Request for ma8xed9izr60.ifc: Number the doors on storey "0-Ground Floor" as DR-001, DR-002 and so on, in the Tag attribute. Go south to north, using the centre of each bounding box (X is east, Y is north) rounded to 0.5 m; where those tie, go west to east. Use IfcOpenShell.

First a look at what the model holds.

```python
import ifcopenshell
import ifcopenshell.util.element
import ifcopenshell.util.placement

model = ifcopenshell.open("ma8xed9izr60.ifc")
print(model.schema)
storey = next(s for s in model.by_type("IfcBuildingStorey") if s.Name == "0-Ground Floor")
doors = [e for e in ifcopenshell.util.element.get_decomposition(storey) if e.is_a("IfcDoor")]
for e in sorted(doors, key=lambda e: e.id()):
    origin = ifcopenshell.util.placement.get_local_placement(e.ObjectPlacement)[:3, 3]
    print(e.id(), e.Tag, e.Name, origin.round(2) + 0.0, sep=" | ")
```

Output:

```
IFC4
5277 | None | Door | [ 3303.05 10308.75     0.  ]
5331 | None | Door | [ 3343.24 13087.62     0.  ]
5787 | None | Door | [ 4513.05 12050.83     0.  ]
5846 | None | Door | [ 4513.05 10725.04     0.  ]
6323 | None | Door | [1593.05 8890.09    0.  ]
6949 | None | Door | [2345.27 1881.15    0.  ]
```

```python
import ifcopenshell
import ifcopenshell.geom
import ifcopenshell.util.element
import ifcopenshell.util.shape

model = ifcopenshell.open("ma8xed9izr60.ifc")
settings = ifcopenshell.geom.settings()
settings.set("use-world-coords", True)


def centre(element):
    shape = ifcopenshell.geom.create_shape(settings, element)
    return ifcopenshell.util.shape.get_bbox_centroid(shape.geometry)


storey = next(s for s in model.by_type("IfcBuildingStorey") if s.Name == "0-Ground Floor")
doors = [e for e in ifcopenshell.util.element.get_decomposition(storey) if e.is_a("IfcDoor")]

# Insertion points can sit at a corner or the storey origin, so sort by the geometry (in metres).
centres = {e: centre(e) for e in doors}
doors.sort(key=lambda e: (round(centres[e][1] / 0.5), centres[e][0]))

for i, e in enumerate(doors, start=1):
    number = f"DR-0{i:02d}"
    e.Tag = number
    print(e.id(), number)

model.write("ma8xed9izr60_edited.ifc")
```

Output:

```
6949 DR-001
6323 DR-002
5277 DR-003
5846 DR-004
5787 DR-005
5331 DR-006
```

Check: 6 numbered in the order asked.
